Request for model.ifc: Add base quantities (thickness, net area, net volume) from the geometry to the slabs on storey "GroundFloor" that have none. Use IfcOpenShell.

First a look at what the model holds.

```python
import ifcopenshell
import ifcopenshell.util.element
import ifcopenshell.util.unit

model = ifcopenshell.open("model.ifc")
print(model.schema)
for unit_type in ("LENGTHUNIT", "AREAUNIT", "VOLUMEUNIT"):
    print(unit_type, ifcopenshell.util.unit.calculate_unit_scale(model, unit_type))
storey = next(s for s in model.by_type("IfcBuildingStorey") if s.Name == "GroundFloor")
slabs = [e for e in ifcopenshell.util.element.get_decomposition(storey) if e.is_a("IfcSlab")]
for e in sorted(slabs, key=lambda e: e.id()):
    print(e.id(), e.is_a(), e.Name, list(ifcopenshell.util.element.get_psets(e, qtos_only=True)), sep=" | ")
```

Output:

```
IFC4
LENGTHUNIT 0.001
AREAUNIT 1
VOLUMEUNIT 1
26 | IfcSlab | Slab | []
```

```python
import ifcopenshell
import ifcopenshell.api.pset
import ifcopenshell.geom
import ifcopenshell.util.element
import ifcopenshell.util.shape
import ifcopenshell.util.unit

model = ifcopenshell.open("model.ifc")
unit_scale = ifcopenshell.util.unit.calculate_unit_scale(model)
area_scale = ifcopenshell.util.unit.calculate_unit_scale(model, "AREAUNIT")
volume_scale = ifcopenshell.util.unit.calculate_unit_scale(model, "VOLUMEUNIT")
settings = ifcopenshell.geom.settings()

storey = next(s for s in model.by_type("IfcBuildingStorey") if s.Name == "GroundFloor")
slabs = [e for e in ifcopenshell.util.element.get_decomposition(storey) if e.is_a("IfcSlab")]

for e in sorted(slabs, key=lambda e: e.id()):
    if ifcopenshell.util.element.get_psets(e, qtos_only=True, should_inherit=False):
        continue
    # Geometry comes back in metres, in the element's own axes.
    shape = ifcopenshell.geom.create_shape(settings, e)
    values = {
        "Width": ifcopenshell.util.shape.get_z(shape.geometry) / unit_scale,
        "NetArea": ifcopenshell.util.shape.get_footprint_area(shape.geometry) / area_scale,
        "NetVolume": ifcopenshell.util.shape.get_volume(shape.geometry) / volume_scale,
    }
    qto = ifcopenshell.api.pset.add_qto(model, product=e, name="Qto_SlabBaseQuantities")
    ifcopenshell.api.pset.edit_qto(model, qto=qto, properties=values)
    print(e.id(), {k: round(v, 3) for k, v in values.items()})

model.write("model_updated.ifc")
```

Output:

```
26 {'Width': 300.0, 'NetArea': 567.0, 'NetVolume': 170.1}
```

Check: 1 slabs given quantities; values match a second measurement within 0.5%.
